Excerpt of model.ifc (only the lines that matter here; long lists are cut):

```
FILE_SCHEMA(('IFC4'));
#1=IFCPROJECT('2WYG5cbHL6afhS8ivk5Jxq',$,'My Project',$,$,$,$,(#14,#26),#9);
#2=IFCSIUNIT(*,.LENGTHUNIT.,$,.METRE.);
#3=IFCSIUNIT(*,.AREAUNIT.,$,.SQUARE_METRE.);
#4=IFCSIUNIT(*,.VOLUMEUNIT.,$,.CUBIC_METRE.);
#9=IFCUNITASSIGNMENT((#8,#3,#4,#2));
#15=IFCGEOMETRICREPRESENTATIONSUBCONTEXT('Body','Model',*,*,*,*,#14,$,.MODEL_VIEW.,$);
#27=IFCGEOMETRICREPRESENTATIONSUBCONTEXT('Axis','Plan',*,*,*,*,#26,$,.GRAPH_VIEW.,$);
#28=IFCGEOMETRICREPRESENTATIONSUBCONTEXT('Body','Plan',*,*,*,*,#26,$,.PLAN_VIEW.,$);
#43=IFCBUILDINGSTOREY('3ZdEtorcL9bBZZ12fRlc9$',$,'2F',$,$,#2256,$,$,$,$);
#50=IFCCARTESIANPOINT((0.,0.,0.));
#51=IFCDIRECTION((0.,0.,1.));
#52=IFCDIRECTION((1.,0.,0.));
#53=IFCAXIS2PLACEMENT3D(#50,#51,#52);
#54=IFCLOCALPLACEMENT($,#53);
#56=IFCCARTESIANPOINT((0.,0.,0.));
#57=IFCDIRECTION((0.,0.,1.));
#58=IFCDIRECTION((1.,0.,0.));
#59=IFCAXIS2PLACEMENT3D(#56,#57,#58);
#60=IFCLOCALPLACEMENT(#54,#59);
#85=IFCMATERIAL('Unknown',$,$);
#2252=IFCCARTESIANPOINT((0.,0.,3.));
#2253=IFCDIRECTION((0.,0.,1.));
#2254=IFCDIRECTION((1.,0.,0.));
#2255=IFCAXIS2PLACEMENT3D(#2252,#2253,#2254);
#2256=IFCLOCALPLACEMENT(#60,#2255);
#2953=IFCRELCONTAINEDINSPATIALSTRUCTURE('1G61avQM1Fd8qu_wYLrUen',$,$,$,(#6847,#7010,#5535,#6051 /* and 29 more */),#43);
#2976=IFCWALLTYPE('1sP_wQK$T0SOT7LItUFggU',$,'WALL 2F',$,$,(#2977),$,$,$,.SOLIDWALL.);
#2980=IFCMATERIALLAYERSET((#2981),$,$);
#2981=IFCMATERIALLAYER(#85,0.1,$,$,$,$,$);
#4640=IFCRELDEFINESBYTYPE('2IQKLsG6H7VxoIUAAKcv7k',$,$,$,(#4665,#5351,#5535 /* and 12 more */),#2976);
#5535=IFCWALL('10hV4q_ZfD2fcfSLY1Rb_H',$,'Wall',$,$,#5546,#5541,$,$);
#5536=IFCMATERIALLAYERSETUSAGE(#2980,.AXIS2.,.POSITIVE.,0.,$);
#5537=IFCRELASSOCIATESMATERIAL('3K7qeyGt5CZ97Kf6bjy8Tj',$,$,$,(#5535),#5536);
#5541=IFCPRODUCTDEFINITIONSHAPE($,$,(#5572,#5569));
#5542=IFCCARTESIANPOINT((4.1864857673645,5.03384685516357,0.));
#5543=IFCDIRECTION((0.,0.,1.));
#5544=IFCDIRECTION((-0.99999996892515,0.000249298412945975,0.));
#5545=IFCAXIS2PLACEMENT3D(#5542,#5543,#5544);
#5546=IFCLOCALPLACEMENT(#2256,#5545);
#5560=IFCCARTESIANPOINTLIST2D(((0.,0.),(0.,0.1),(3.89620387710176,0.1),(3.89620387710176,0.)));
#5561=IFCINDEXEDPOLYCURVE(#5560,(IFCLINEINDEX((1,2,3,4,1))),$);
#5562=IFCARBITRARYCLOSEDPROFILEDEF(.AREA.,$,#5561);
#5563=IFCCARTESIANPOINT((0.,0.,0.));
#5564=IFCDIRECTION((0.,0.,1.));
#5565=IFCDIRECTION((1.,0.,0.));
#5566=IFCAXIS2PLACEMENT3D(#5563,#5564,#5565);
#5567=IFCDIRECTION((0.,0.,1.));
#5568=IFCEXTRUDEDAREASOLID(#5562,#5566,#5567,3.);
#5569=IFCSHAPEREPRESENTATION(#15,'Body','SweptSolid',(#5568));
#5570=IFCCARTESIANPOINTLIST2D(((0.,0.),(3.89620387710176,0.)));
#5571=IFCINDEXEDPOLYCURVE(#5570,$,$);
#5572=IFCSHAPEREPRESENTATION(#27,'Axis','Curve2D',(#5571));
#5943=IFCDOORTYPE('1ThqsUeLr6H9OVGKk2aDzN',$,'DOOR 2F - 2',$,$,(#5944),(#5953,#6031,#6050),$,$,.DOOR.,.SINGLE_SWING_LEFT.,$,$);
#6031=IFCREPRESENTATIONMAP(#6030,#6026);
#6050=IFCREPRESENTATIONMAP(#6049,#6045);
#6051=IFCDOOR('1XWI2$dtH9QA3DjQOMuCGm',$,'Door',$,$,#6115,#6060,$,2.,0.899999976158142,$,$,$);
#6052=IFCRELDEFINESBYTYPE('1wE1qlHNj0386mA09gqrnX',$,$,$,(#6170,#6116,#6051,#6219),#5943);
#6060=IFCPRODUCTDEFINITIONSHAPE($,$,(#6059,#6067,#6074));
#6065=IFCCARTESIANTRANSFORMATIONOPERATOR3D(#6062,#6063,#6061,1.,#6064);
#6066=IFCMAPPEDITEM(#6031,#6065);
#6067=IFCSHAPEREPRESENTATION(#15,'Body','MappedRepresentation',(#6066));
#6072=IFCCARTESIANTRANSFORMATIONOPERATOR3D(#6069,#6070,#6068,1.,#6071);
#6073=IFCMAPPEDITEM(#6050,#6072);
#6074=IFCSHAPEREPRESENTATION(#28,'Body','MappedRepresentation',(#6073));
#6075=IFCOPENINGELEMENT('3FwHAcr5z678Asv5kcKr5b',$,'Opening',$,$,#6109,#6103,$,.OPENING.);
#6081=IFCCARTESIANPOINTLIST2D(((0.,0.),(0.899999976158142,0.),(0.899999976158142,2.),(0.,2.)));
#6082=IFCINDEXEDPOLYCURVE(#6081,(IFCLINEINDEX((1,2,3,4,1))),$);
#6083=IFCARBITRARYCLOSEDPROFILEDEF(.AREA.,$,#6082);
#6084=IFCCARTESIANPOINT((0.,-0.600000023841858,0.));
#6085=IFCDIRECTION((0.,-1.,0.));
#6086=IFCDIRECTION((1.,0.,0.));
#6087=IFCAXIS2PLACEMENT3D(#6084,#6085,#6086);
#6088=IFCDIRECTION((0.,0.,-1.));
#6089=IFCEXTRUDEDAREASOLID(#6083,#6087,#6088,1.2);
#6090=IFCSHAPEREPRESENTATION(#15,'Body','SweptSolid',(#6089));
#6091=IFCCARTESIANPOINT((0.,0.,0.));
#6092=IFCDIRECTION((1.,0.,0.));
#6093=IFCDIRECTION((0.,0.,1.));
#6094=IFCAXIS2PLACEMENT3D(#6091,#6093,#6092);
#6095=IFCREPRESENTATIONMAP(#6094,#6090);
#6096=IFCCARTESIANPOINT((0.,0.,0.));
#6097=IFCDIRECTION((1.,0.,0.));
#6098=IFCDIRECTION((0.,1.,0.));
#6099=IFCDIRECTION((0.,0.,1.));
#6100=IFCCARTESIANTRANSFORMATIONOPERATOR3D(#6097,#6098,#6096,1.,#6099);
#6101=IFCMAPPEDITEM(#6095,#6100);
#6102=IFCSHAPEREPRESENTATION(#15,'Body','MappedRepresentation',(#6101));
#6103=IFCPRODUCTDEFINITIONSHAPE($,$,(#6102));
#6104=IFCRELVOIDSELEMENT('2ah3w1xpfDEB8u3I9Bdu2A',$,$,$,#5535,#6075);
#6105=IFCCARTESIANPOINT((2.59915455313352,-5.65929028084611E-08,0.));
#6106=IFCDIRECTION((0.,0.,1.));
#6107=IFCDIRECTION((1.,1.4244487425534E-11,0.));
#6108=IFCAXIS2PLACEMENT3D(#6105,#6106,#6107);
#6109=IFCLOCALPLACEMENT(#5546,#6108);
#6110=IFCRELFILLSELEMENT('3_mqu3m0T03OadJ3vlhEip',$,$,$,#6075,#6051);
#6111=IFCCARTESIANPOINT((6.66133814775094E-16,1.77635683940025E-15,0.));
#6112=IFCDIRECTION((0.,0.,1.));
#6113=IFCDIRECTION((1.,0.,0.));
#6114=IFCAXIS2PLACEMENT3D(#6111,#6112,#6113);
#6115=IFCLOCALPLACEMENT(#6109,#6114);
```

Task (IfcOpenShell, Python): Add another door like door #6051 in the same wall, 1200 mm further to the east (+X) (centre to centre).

```python
import ifcopenshell
import ifcopenshell.api.feature
import ifcopenshell.api.geometry
import ifcopenshell.api.root
import ifcopenshell.geom
import ifcopenshell.util.element
import ifcopenshell.util.placement
import ifcopenshell.util.shape
import ifcopenshell.util.unit

model = ifcopenshell.open("model.ifc")
unit_scale = ifcopenshell.util.unit.calculate_unit_scale(model)
settings = ifcopenshell.geom.settings()


def volume(element):
    """Net volume in cubic metres, openings subtracted."""
    shape = ifcopenshell.geom.create_shape(settings, element)
    return ifcopenshell.util.shape.get_volume(shape.geometry)


door = model.by_guid("1XWI2$dtH9QA3DjQOMuCGm")
opening = door.FillsVoids[0].RelatingOpeningElement
wall = opening.VoidsElements[0].RelatingBuildingElement
before = volume(wall)
shift = ifcopenshell.util.placement.get_local_placement(wall.ObjectPlacement)[:3, 0] * -1.2 / unit_scale

# copy_class copies the void relationship, type, container and properties, but no geometry.
new_opening = ifcopenshell.api.root.copy_class(model, product=opening)
new_opening.Representation = ifcopenshell.util.element.copy_deep(
    model, opening.Representation, exclude=["IfcGeometricRepresentationContext", "IfcRepresentationMap"]
)
new_door = ifcopenshell.api.root.copy_class(model, product=door)
new_door.Representation = ifcopenshell.util.element.copy_deep(
    model, door.Representation, exclude=["IfcGeometricRepresentationContext", "IfcRepresentationMap"]
)
ifcopenshell.api.feature.add_filling(model, opening=new_opening, element=new_door)

for old, new in ((opening, new_opening), (door, new_door)):
    matrix = ifcopenshell.util.placement.get_local_placement(old.ObjectPlacement)
    matrix[:3, 3] += shift
    ifcopenshell.api.geometry.edit_object_placement(model, product=new, matrix=matrix, is_si=False)

after = volume(wall)

print(f"wall volume {before:.3f} -> {after:.3f} m3")

model.write("model_v2.ifc")
```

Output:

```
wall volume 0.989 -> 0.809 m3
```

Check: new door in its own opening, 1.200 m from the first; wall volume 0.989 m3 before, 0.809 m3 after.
